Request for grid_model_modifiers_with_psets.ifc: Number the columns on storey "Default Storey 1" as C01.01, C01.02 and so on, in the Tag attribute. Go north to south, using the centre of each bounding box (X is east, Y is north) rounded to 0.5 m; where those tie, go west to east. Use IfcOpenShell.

First a look at what the model holds.

```python
import ifcopenshell
import ifcopenshell.util.element
import ifcopenshell.util.placement

model = ifcopenshell.open("grid_model_modifiers_with_psets.ifc")
print(model.schema)
storey = next(s for s in model.by_type("IfcBuildingStorey") if s.Name == "Default Storey 1")
columns = [e for e in ifcopenshell.util.element.get_decomposition(storey) if e.is_a("IfcColumn")]
for e in sorted(columns, key=lambda e: e.id()):
    origin = ifcopenshell.util.placement.get_local_placement(e.ObjectPlacement)[:3, 3]
    print(e.id(), e.Tag, e.Name, origin.round(2) + 0.0, sep=" | ")
```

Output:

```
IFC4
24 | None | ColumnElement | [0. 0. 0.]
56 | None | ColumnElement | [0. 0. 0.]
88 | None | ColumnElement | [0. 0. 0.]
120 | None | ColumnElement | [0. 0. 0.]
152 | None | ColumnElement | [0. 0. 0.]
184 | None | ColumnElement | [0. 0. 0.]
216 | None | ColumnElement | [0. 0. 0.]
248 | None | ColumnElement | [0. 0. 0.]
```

```python
import ifcopenshell
import ifcopenshell.geom
import ifcopenshell.util.element
import ifcopenshell.util.shape

model = ifcopenshell.open("grid_model_modifiers_with_psets.ifc")
settings = ifcopenshell.geom.settings()
settings.set("use-world-coords", True)


def centre(element):
    shape = ifcopenshell.geom.create_shape(settings, element)
    return ifcopenshell.util.shape.get_bbox_centroid(shape.geometry)


storey = next(s for s in model.by_type("IfcBuildingStorey") if s.Name == "Default Storey 1")
columns = [e for e in ifcopenshell.util.element.get_decomposition(storey) if e.is_a("IfcColumn")]

# Insertion points can sit at a corner or the storey origin, so sort by the geometry (in metres).
centres = {e: centre(e) for e in columns}
columns.sort(key=lambda e: (-round(centres[e][1] / 0.5), centres[e][0]))

for i, e in enumerate(columns, start=1):
    number = f"C01.{i:02d}"
    e.Tag = number
    print(e.id(), number)

model.write("grid_model_modifiers_with_psets_v2.ifc")
```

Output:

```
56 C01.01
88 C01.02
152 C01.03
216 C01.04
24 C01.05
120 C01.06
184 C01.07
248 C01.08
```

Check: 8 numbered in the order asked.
